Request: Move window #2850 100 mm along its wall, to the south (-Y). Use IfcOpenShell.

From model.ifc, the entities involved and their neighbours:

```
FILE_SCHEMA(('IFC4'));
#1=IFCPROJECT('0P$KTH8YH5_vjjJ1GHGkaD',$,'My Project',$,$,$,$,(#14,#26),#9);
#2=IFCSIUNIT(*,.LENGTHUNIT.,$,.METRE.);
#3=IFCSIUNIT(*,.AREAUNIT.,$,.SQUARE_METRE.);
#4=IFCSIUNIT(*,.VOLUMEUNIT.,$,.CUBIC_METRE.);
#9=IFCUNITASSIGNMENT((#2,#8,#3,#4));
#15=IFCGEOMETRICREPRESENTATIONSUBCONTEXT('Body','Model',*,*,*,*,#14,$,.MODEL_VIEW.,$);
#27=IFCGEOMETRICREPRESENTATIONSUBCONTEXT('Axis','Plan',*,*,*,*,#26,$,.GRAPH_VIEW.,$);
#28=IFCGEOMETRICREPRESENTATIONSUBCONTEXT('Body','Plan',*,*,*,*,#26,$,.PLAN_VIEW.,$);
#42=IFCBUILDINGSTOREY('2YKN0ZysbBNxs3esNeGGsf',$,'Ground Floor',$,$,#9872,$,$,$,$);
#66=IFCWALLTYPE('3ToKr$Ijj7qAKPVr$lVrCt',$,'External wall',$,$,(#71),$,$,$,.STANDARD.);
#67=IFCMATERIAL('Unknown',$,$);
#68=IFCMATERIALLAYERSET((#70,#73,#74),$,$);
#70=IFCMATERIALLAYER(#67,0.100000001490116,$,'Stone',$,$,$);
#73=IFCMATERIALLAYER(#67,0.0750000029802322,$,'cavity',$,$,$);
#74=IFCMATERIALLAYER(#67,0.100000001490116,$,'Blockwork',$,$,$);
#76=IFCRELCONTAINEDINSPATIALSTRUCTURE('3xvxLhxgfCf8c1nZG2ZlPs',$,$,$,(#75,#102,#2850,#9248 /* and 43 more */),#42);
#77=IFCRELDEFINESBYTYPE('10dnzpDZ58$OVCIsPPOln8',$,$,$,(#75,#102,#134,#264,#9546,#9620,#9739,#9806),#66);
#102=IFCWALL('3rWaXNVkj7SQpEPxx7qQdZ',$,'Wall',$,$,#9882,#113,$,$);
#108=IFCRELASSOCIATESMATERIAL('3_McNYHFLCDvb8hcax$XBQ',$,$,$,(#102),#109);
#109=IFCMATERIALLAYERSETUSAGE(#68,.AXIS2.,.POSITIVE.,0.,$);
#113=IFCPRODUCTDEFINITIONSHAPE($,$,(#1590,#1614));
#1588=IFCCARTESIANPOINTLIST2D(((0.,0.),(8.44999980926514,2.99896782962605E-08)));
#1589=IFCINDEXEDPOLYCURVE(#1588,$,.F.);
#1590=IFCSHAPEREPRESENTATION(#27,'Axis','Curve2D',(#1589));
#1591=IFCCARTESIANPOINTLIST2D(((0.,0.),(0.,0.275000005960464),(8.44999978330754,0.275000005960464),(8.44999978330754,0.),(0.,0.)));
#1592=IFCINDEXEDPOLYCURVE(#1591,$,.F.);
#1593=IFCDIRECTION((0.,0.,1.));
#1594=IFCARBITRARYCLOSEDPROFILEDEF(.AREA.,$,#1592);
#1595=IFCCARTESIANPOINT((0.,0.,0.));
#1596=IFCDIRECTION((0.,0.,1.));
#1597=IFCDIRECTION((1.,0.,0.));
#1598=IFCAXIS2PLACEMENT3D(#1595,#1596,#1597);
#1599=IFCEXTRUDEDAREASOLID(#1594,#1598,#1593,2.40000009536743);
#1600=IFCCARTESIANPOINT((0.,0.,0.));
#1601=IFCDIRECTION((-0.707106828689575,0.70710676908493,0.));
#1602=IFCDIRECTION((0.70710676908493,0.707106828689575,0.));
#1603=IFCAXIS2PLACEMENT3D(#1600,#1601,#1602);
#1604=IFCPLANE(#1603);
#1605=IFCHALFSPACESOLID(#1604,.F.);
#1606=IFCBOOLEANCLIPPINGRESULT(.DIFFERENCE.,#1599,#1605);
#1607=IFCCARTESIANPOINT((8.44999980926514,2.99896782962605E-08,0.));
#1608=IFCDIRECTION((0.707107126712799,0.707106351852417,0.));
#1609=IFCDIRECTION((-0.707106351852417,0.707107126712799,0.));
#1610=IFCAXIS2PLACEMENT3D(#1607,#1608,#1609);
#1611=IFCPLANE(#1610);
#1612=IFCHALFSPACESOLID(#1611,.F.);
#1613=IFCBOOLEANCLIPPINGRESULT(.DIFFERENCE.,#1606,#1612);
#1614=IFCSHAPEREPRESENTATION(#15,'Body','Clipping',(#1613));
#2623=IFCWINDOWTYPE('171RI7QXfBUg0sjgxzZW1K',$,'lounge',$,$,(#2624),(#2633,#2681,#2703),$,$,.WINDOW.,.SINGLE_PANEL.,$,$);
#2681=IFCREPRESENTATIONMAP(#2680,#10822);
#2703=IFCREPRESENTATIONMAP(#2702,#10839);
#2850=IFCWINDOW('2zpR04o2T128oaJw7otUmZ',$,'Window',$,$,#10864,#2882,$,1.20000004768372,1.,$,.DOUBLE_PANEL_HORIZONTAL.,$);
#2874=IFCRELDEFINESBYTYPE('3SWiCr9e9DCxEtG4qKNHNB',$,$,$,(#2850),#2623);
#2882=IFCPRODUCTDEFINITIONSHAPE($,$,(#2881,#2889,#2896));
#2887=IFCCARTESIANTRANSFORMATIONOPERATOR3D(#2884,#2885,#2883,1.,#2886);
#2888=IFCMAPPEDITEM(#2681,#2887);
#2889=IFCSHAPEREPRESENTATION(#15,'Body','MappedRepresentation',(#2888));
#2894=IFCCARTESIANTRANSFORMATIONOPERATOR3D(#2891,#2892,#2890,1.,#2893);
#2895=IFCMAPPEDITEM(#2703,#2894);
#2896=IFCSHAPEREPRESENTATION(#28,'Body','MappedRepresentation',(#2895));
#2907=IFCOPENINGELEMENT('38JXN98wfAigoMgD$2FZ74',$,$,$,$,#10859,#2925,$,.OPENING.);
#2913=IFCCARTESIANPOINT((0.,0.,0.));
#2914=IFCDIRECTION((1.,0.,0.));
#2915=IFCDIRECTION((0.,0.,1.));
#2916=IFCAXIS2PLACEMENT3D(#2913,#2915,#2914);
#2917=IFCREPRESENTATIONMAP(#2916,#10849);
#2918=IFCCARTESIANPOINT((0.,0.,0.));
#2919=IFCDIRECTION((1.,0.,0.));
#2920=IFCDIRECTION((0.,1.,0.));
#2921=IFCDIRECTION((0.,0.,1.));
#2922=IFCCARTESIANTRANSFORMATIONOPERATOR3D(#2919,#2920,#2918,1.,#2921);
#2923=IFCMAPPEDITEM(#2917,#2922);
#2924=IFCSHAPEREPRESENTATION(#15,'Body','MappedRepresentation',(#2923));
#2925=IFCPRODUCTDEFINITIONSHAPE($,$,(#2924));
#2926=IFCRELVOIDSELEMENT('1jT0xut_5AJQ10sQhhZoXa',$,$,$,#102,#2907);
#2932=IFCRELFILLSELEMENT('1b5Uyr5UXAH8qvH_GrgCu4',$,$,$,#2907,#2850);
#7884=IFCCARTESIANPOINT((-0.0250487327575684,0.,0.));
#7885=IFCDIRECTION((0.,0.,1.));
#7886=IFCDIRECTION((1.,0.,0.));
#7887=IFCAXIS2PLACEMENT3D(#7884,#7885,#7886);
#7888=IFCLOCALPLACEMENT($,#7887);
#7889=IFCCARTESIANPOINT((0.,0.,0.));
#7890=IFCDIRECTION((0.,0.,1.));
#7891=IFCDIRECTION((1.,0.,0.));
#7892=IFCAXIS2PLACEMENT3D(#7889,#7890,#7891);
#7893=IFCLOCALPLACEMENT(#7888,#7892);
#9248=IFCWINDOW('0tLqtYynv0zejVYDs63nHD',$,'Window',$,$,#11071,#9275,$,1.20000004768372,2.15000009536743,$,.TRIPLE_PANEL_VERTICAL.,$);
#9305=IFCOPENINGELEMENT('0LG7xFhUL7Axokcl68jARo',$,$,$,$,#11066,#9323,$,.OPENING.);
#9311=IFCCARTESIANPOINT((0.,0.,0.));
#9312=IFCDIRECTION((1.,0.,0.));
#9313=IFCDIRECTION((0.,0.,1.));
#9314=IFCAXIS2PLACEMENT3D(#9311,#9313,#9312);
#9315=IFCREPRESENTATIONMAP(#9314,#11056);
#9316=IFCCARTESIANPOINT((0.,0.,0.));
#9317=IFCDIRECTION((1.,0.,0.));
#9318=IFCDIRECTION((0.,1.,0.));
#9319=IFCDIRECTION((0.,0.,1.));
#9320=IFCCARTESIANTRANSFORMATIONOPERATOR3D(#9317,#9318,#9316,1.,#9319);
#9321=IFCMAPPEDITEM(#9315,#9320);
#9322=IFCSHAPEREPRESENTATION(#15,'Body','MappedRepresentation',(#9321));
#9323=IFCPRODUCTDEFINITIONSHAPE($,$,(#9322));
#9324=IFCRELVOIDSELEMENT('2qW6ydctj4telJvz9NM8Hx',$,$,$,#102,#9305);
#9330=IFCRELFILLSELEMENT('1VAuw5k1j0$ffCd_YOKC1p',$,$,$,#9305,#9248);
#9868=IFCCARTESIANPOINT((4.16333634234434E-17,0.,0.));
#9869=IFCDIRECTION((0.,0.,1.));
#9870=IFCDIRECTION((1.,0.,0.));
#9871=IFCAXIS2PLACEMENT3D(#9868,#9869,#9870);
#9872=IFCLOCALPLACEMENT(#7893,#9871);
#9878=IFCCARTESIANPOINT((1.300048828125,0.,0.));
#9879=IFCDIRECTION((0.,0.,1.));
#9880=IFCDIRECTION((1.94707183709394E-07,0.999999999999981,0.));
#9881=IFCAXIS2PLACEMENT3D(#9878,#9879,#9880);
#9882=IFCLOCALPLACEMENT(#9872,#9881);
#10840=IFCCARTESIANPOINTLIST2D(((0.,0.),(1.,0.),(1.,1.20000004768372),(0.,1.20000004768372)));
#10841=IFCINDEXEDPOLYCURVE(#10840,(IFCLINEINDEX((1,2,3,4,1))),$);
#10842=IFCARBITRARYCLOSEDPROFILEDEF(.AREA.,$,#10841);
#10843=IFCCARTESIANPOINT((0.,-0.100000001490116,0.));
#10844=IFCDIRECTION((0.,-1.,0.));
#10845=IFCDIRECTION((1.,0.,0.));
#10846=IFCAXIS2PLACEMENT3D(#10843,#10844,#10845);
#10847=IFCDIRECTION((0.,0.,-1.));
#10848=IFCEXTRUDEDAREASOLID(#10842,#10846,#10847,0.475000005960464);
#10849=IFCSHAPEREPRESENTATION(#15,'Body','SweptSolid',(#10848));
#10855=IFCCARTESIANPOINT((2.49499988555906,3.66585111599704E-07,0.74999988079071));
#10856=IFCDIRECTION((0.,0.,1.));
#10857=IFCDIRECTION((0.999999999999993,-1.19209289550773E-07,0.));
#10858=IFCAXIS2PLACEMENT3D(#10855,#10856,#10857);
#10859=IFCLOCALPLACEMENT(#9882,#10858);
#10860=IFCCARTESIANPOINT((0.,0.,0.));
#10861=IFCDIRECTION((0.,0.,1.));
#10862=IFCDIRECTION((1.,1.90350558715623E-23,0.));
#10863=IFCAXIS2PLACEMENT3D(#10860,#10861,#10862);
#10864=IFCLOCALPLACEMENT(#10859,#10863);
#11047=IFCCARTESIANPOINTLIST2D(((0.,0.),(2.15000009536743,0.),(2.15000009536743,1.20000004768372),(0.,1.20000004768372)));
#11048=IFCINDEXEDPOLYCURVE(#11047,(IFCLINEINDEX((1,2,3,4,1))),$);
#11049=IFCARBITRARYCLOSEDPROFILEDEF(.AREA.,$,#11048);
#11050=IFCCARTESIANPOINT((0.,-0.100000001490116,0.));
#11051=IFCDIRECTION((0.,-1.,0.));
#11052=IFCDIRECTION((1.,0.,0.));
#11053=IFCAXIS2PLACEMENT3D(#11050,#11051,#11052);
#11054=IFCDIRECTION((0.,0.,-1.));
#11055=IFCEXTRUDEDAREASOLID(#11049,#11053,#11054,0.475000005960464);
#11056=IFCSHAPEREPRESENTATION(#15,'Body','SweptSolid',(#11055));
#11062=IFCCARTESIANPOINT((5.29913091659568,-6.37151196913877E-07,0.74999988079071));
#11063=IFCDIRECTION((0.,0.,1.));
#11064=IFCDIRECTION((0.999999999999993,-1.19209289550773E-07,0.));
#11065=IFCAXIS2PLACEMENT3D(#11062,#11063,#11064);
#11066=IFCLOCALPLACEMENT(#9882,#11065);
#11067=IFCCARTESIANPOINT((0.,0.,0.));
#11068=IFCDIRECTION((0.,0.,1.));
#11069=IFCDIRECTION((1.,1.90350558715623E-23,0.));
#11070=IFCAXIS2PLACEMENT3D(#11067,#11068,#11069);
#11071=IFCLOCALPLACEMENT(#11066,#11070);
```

```python
import ifcopenshell
import ifcopenshell.api.geometry
import ifcopenshell.util.placement
import ifcopenshell.util.unit

model = ifcopenshell.open("model.ifc")
unit_scale = ifcopenshell.util.unit.calculate_unit_scale(model)

window = model.by_guid("2zpR04o2T128oaJw7otUmZ")
opening = window.FillsVoids[0].RelatingOpeningElement
wall = opening.VoidsElements[0].RelatingBuildingElement

wall_matrix = ifcopenshell.util.placement.get_local_placement(wall.ObjectPlacement)
shift = wall_matrix[:3, 0] * -0.1 / unit_scale
before = ifcopenshell.util.placement.get_local_placement(window.ObjectPlacement)[:3, 3].copy()

# The window is placed relative to its opening, so it follows when the opening moves.
matrix = ifcopenshell.util.placement.get_local_placement(opening.ObjectPlacement)
matrix[:3, 3] += shift
ifcopenshell.api.geometry.edit_object_placement(
    model, product=opening, matrix=matrix, is_si=False, should_transform_children=True
)

after = ifcopenshell.util.placement.get_local_placement(window.ObjectPlacement)[:3, 3]
print("window moved by", (after - before).round(3) + 0.0)

model.write("model_updated.ifc")
```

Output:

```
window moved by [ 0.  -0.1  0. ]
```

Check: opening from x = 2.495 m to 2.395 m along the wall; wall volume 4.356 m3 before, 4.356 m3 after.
